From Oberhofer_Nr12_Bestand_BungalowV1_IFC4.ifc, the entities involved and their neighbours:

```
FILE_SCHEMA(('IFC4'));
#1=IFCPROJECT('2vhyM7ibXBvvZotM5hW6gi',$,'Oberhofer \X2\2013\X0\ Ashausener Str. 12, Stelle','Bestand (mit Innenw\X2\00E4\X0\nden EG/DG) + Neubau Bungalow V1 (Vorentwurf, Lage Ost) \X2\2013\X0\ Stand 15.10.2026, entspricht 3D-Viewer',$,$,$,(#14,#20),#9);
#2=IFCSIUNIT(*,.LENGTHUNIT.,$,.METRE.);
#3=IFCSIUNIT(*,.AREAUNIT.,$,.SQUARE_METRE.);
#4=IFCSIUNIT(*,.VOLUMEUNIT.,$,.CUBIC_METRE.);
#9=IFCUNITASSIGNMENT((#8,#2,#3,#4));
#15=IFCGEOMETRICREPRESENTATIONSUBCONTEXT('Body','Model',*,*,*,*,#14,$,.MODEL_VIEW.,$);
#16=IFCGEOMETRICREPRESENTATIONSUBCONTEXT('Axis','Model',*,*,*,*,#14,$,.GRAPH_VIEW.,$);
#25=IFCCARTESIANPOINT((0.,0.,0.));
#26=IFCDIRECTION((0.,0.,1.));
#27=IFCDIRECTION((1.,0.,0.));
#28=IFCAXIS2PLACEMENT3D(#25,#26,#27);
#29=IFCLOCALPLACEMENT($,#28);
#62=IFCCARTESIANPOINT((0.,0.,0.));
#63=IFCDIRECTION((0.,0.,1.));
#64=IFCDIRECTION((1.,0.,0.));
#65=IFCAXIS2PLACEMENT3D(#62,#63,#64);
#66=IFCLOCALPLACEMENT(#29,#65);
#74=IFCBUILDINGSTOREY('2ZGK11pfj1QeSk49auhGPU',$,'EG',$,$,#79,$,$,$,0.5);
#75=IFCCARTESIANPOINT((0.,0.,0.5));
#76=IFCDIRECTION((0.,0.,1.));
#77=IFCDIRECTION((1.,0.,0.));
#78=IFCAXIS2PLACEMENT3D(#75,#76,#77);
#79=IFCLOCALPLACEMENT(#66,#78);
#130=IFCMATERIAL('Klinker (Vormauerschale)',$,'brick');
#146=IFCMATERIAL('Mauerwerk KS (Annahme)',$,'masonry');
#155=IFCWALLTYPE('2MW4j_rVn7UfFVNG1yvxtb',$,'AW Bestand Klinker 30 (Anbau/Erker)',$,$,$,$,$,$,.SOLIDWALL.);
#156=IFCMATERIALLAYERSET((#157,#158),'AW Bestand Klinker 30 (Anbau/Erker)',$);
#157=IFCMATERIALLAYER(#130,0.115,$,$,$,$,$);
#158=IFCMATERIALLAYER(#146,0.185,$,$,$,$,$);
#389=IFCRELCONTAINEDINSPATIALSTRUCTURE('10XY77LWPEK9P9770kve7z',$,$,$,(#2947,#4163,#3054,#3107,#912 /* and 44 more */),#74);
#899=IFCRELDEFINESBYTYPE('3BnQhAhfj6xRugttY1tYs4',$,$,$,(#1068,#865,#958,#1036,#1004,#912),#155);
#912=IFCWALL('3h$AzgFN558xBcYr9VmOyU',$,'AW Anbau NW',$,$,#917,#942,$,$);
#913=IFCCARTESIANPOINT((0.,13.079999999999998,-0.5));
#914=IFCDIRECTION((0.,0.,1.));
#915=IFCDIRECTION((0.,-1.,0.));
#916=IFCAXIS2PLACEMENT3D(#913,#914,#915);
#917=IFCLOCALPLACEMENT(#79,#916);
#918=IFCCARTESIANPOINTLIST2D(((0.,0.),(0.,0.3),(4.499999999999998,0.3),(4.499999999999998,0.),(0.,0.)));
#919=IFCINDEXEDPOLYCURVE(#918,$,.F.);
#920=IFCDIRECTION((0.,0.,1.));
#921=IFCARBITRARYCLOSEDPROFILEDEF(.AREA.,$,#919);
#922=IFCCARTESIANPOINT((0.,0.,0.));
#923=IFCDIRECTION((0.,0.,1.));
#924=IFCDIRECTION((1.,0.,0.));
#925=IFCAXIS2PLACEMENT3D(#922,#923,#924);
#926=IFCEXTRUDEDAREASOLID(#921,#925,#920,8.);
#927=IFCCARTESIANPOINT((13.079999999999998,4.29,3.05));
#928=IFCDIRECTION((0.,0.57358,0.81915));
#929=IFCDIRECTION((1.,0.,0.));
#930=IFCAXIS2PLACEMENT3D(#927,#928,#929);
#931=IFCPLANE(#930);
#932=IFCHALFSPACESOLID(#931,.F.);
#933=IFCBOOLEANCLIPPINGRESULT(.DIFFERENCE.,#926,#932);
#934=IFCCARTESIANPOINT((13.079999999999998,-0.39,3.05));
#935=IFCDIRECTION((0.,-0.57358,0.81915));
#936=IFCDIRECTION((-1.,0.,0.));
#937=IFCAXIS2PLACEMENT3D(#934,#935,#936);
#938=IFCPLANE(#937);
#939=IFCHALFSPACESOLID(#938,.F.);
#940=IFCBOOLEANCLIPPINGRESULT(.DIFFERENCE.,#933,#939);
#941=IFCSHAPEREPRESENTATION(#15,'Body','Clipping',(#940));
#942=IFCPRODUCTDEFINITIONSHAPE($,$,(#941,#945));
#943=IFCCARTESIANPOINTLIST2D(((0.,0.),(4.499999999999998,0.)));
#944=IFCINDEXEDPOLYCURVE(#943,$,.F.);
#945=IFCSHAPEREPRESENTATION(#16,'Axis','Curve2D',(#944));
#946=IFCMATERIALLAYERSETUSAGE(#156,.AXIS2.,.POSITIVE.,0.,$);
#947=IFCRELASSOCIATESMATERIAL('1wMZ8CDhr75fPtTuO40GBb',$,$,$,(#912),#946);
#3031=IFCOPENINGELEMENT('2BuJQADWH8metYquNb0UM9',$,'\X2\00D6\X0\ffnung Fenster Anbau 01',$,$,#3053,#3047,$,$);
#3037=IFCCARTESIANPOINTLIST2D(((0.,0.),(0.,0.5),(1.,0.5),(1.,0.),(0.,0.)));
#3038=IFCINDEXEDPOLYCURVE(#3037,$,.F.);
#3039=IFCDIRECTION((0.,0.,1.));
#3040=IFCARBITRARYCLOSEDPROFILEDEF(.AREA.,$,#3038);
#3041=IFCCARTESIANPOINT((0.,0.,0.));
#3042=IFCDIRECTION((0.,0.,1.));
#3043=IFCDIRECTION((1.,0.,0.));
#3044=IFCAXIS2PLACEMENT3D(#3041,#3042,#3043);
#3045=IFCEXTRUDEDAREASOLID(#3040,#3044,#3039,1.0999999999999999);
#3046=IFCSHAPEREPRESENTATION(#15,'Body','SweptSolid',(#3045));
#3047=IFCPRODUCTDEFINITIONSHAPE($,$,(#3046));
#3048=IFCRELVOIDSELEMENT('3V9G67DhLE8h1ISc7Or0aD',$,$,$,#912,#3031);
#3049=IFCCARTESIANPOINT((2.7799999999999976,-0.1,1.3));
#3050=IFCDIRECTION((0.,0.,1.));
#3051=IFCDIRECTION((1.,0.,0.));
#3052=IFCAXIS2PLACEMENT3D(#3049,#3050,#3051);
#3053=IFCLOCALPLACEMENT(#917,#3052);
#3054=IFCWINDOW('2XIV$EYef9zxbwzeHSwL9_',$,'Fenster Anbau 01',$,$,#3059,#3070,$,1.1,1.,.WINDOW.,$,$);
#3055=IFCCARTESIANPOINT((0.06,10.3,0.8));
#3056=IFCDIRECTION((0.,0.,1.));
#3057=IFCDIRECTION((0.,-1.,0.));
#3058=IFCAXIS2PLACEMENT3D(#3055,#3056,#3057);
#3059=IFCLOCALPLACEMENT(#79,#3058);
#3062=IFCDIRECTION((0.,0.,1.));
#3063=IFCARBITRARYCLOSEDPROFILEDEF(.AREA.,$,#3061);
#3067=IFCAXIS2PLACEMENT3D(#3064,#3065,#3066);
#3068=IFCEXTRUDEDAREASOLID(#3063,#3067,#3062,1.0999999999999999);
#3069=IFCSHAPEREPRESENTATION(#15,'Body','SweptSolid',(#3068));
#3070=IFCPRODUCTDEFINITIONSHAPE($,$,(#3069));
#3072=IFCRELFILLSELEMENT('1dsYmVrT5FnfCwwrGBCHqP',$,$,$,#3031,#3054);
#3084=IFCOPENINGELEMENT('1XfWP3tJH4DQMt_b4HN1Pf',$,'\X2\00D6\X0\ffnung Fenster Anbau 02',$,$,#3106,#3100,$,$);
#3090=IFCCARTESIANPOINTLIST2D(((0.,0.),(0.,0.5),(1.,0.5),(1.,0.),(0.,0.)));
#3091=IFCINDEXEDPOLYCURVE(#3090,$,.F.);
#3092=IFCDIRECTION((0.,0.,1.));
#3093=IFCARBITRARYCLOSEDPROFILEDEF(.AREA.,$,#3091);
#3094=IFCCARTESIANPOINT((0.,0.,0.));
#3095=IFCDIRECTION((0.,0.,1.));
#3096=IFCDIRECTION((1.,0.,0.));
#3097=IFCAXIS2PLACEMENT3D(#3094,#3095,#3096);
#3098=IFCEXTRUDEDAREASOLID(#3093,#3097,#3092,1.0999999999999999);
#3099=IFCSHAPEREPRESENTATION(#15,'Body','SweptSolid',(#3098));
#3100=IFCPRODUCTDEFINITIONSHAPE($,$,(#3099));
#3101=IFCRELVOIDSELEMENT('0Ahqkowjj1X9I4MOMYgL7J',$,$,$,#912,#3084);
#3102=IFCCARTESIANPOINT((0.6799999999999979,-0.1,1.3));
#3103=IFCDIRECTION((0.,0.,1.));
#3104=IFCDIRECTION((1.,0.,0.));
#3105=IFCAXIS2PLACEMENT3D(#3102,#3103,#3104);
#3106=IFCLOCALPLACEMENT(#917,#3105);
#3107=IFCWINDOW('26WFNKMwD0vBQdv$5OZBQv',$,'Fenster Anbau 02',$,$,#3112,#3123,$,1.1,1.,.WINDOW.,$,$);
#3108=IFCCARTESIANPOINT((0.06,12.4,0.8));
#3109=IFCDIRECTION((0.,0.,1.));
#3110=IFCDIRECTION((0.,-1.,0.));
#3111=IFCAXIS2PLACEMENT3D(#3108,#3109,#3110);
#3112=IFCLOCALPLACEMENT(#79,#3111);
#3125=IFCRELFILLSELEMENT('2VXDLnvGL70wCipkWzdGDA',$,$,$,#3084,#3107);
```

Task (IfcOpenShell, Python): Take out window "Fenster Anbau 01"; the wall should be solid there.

```python
import ifcopenshell
import ifcopenshell.api.feature
import ifcopenshell.api.root
import ifcopenshell.geom
import ifcopenshell.util.shape

model = ifcopenshell.open("Oberhofer_Nr12_Bestand_BungalowV1_IFC4.ifc")
settings = ifcopenshell.geom.settings()


def volume(element):
    """Net volume in cubic metres, openings subtracted."""
    shape = ifcopenshell.geom.create_shape(settings, element)
    return ifcopenshell.util.shape.get_volume(shape.geometry)


window = model.by_guid("2XIV$EYef9zxbwzeHSwL9_")
opening = window.FillsVoids[0].RelatingOpeningElement
wall = opening.VoidsElements[0].RelatingBuildingElement
before = volume(wall)

ifcopenshell.api.root.remove_product(model, product=window)
ifcopenshell.api.feature.remove_feature(model, feature=opening)

after = volume(wall)

print(f"wall volume {before:.3f} -> {after:.3f} m3")

model.write("Oberhofer_Nr12_Bestand_BungalowV1_IFC4_updated.ifc")
```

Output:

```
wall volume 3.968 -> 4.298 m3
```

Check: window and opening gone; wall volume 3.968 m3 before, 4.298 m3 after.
